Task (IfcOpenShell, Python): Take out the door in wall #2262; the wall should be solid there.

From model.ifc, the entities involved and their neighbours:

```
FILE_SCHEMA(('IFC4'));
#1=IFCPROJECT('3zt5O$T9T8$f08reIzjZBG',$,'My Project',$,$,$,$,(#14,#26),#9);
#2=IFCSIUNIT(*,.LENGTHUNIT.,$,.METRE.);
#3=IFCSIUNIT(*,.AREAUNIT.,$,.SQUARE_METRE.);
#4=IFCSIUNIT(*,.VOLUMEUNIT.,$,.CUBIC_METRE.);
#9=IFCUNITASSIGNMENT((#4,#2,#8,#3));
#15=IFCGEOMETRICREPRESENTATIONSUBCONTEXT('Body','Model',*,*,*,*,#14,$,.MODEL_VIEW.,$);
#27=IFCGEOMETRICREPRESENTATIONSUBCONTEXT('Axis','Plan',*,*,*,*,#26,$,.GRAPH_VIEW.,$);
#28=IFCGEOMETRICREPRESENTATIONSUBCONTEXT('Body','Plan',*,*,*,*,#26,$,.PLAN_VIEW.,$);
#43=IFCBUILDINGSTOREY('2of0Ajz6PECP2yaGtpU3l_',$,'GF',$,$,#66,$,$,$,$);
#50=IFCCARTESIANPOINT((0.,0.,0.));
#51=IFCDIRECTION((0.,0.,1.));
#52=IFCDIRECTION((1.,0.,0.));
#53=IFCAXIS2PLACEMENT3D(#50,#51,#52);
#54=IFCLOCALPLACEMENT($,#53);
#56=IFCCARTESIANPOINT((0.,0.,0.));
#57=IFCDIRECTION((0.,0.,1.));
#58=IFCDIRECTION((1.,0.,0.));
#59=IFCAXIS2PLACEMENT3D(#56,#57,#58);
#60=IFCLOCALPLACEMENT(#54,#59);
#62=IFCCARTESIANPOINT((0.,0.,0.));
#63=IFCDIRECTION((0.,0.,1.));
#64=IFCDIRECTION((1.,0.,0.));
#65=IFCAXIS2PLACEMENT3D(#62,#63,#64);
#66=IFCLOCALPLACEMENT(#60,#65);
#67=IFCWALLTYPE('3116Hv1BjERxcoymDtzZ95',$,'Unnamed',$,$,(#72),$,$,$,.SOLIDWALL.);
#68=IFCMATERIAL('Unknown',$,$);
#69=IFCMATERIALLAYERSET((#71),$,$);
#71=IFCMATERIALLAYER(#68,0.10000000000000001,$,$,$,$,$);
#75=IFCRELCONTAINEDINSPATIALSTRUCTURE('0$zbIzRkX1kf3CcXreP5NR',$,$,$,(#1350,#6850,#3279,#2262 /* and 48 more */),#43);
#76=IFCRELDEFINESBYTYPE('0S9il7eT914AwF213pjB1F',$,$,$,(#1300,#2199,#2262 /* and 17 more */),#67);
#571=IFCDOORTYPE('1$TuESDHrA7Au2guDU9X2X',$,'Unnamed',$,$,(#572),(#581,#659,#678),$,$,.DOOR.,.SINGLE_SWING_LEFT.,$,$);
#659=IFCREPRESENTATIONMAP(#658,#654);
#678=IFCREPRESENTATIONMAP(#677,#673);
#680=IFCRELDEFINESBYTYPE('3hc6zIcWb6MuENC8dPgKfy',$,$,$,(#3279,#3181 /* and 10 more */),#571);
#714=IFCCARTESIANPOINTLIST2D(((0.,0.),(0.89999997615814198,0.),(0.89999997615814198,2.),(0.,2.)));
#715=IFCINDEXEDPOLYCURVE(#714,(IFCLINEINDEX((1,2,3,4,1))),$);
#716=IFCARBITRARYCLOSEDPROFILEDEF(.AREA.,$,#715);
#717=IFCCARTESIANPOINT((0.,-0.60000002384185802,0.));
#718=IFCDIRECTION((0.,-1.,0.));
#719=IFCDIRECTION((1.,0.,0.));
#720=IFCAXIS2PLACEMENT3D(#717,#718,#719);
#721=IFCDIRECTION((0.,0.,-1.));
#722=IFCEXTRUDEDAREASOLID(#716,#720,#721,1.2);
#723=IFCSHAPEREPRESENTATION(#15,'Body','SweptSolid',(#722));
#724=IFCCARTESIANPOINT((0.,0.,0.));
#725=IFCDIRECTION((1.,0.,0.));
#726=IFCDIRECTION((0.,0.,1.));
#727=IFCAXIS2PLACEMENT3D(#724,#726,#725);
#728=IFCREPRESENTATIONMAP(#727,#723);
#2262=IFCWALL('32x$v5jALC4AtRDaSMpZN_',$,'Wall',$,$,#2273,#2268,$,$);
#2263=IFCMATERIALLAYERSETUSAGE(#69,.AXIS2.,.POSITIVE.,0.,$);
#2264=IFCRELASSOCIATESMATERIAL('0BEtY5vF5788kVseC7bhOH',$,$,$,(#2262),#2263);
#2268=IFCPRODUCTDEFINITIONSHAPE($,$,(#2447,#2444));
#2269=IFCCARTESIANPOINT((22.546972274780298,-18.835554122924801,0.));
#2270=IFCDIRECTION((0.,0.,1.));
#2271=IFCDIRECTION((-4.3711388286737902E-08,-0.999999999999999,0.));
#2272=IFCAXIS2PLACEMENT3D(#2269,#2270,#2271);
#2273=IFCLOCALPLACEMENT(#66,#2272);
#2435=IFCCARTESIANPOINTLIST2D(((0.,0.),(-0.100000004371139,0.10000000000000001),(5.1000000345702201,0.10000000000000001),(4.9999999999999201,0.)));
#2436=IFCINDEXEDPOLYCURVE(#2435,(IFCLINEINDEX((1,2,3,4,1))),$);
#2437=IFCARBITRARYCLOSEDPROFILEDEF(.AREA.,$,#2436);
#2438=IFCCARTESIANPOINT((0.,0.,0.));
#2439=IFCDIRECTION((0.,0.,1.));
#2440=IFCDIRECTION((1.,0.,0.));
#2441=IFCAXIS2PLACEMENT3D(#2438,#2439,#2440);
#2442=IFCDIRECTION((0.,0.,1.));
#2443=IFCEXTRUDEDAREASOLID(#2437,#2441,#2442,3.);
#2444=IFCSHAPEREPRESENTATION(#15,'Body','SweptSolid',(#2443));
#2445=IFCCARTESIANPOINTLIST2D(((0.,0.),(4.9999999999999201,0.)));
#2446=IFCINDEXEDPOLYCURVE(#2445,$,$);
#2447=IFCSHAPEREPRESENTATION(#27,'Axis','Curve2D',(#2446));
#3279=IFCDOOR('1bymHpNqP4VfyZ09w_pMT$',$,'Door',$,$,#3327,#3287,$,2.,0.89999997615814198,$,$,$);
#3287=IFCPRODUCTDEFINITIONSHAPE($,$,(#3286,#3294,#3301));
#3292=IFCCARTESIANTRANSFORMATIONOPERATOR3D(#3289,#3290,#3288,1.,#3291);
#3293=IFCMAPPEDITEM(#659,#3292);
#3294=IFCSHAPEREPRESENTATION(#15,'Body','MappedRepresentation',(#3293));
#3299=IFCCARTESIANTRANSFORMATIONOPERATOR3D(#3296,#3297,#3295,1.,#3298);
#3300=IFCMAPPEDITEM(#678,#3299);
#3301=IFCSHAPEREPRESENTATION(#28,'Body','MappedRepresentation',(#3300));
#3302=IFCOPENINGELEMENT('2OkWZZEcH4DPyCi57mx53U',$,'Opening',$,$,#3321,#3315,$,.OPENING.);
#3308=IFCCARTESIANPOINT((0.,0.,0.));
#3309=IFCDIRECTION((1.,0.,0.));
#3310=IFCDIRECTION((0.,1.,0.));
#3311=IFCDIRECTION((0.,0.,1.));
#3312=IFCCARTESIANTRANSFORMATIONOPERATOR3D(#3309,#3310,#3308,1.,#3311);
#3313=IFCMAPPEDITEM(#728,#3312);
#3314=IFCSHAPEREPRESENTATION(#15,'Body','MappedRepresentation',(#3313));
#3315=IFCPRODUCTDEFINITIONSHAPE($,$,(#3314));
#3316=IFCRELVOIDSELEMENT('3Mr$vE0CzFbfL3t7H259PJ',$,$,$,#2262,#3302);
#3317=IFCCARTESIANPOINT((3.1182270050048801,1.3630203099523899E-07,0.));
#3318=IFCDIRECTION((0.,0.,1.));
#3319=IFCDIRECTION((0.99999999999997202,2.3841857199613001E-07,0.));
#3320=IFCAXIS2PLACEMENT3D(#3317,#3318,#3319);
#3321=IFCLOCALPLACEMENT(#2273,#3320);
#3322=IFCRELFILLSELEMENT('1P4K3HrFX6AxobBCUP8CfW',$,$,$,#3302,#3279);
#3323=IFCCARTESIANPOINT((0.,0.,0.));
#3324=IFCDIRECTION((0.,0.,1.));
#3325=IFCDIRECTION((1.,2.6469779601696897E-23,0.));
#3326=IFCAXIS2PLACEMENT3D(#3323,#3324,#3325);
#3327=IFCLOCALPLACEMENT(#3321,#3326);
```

```python
import ifcopenshell
import ifcopenshell.api.feature
import ifcopenshell.api.root
import ifcopenshell.geom
import ifcopenshell.util.shape

model = ifcopenshell.open("model.ifc")
settings = ifcopenshell.geom.settings()


def volume(element):
    """Net volume in cubic metres, openings subtracted."""
    shape = ifcopenshell.geom.create_shape(settings, element)
    return ifcopenshell.util.shape.get_volume(shape.geometry)


door = model.by_guid("1bymHpNqP4VfyZ09w_pMT$")
opening = door.FillsVoids[0].RelatingOpeningElement
wall = opening.VoidsElements[0].RelatingBuildingElement
before = volume(wall)

ifcopenshell.api.root.remove_product(model, product=door)
ifcopenshell.api.feature.remove_feature(model, feature=opening)

after = volume(wall)

print(f"wall volume {before:.3f} -> {after:.3f} m3")

model.write("model_edited.ifc")
```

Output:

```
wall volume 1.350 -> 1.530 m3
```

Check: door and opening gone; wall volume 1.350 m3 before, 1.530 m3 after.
